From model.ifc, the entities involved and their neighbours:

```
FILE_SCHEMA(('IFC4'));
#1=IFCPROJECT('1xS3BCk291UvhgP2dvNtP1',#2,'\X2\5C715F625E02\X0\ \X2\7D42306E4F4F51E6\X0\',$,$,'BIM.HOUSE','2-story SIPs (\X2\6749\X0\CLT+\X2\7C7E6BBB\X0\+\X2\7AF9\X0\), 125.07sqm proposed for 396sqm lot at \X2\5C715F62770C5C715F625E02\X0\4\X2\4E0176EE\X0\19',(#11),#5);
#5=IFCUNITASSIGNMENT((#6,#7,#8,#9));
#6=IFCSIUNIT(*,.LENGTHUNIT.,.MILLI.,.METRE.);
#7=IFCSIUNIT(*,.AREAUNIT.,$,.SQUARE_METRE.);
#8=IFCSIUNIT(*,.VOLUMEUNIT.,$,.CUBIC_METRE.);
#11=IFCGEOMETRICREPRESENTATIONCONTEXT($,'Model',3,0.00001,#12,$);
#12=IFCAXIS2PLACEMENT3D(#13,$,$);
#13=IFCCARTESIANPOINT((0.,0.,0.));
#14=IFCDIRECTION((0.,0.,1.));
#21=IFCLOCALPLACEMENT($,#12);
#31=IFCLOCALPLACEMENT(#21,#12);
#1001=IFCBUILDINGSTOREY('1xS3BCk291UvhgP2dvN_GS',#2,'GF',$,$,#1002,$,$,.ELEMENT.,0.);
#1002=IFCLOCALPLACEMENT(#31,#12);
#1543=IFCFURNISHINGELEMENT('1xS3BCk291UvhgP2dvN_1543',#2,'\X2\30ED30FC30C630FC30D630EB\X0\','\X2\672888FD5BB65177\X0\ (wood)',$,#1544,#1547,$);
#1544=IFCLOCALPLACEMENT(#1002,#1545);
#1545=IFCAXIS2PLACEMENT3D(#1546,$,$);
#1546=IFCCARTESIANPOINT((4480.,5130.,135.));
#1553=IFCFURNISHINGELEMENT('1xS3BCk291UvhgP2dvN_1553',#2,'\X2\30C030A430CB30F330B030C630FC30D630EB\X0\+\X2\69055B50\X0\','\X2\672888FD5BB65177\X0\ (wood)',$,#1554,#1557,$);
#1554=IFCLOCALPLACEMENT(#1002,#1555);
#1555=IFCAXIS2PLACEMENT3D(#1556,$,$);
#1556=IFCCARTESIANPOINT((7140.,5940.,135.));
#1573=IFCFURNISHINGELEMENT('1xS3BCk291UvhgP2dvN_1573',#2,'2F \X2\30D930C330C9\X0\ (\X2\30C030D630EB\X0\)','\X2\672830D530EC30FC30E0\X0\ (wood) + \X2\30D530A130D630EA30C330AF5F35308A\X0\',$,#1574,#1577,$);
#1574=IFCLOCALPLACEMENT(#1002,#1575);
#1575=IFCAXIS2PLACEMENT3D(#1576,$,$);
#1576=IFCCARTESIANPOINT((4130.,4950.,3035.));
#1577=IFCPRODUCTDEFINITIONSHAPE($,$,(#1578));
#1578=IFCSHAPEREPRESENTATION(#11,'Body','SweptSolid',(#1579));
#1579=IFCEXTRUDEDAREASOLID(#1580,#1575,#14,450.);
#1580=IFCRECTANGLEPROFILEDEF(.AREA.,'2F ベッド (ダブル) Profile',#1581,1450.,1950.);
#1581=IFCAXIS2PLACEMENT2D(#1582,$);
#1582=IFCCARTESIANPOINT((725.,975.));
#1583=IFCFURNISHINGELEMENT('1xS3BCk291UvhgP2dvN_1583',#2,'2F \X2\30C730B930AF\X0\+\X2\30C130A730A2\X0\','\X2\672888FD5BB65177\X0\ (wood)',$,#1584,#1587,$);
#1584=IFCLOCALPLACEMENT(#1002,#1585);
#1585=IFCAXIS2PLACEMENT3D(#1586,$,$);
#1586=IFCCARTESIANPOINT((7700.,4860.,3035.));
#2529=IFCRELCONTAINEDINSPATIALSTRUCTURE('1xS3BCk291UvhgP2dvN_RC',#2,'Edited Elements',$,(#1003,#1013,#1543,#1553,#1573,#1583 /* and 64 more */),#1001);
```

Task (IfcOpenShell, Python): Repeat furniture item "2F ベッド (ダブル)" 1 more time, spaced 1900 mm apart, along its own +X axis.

```python
import ifcopenshell
import ifcopenshell.api.geometry
import ifcopenshell.api.root
import ifcopenshell.util.element
import ifcopenshell.util.placement

model = ifcopenshell.open("model.ifc")


def reuse_history(source, copy):
    """copy_class also copies each property set's owner history, people and application; keep the originals."""
    for rel in copy.IsDefinedBy:
        if rel.is_a("IfcRelDefinesByProperties") and (history := rel.RelatingPropertyDefinition.OwnerHistory):
            rel.RelatingPropertyDefinition.OwnerHistory = source.OwnerHistory
            ifcopenshell.util.element.remove_deep2(model, history)


source = model.by_id(1573)
base = ifcopenshell.util.placement.get_local_placement(source.ObjectPlacement)
step = base[:3, 0] * 1900.0

for i in range(1, 2):
    copy = ifcopenshell.api.root.copy_class(model, product=source)
    copy.Representation = ifcopenshell.util.element.copy_deep(
        model, source.Representation, exclude=["IfcGeometricRepresentationContext", "IfcRepresentationMap"]
    )
    reuse_history(source, copy)
    matrix = base.copy()
    matrix[:3, 3] += i * step
    print("added at", matrix[:3, 3].round(3) + 0.0)
    ifcopenshell.api.geometry.edit_object_placement(model, product=copy, matrix=matrix, is_si=False)

model.write("model_updated.ifc")
```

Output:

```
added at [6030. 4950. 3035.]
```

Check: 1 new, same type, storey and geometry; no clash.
